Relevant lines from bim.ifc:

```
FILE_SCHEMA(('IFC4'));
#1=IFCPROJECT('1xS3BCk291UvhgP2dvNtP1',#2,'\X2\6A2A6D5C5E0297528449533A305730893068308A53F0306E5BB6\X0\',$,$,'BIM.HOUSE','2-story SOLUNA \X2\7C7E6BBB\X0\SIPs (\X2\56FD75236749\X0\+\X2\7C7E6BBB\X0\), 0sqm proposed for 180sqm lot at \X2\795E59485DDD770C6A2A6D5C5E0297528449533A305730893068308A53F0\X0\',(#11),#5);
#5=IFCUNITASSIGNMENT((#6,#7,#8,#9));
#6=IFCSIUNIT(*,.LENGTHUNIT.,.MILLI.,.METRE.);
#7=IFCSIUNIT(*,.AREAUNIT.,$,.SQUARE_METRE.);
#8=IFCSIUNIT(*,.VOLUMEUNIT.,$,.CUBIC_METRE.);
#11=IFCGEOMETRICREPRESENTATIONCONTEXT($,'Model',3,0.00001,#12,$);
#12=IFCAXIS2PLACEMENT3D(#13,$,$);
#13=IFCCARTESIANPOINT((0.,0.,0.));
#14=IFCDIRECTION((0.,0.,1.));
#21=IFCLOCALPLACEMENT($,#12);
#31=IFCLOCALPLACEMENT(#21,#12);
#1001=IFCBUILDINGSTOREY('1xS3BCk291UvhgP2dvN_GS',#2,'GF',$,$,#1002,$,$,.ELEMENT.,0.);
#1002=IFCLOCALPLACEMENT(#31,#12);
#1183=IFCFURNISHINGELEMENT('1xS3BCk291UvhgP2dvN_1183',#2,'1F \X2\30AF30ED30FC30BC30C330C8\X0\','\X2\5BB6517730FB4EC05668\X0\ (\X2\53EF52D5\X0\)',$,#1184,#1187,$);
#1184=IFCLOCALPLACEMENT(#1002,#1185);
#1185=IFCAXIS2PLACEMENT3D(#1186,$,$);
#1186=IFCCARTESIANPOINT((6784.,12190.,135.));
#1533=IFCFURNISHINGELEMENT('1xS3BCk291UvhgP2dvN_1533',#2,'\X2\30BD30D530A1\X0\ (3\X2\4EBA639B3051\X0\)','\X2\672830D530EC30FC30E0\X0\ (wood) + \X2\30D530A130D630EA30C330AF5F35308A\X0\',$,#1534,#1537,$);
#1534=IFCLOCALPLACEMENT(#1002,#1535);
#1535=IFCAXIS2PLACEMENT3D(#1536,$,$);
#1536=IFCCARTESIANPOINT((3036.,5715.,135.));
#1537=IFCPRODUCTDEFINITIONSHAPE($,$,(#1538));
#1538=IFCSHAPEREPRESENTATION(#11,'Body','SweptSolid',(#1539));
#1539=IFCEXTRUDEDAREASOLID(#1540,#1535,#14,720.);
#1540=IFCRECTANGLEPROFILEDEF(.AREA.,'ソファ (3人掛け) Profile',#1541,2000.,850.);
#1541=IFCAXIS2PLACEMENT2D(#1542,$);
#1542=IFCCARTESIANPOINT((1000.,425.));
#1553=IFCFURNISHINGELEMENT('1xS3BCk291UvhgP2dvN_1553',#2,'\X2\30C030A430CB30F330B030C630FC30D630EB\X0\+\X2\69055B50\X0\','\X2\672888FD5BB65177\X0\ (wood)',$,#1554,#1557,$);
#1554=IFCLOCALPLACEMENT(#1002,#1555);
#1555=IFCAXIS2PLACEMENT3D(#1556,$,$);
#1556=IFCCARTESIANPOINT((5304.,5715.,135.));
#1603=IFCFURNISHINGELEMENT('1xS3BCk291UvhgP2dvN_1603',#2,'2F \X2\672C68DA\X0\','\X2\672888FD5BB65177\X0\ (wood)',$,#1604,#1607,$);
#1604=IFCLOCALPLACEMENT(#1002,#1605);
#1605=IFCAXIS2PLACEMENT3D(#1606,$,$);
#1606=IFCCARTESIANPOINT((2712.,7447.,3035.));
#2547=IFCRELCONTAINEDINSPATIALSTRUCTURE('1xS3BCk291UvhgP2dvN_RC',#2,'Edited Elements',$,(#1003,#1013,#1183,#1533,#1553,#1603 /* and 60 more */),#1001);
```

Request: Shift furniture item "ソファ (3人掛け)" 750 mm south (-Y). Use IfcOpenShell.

```python
import ifcopenshell
import ifcopenshell.api.geometry
import ifcopenshell.util.placement

model = ifcopenshell.open("bim.ifc")

item = model.by_guid("1xS3BCk291UvhgP2dvN_1533")
matrix = ifcopenshell.util.placement.get_local_placement(item.ObjectPlacement)
matrix[1, 3] -= 750.0
ifcopenshell.api.geometry.edit_object_placement(model, product=item, matrix=matrix, is_si=False)

print(ifcopenshell.util.placement.get_local_placement(item.ObjectPlacement).round(3) + 0.0)

model.write("bim_rev.ifc")
```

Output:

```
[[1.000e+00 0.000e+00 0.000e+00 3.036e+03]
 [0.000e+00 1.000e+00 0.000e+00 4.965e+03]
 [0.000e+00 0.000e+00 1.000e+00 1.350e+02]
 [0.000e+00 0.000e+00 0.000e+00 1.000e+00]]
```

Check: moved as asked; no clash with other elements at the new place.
